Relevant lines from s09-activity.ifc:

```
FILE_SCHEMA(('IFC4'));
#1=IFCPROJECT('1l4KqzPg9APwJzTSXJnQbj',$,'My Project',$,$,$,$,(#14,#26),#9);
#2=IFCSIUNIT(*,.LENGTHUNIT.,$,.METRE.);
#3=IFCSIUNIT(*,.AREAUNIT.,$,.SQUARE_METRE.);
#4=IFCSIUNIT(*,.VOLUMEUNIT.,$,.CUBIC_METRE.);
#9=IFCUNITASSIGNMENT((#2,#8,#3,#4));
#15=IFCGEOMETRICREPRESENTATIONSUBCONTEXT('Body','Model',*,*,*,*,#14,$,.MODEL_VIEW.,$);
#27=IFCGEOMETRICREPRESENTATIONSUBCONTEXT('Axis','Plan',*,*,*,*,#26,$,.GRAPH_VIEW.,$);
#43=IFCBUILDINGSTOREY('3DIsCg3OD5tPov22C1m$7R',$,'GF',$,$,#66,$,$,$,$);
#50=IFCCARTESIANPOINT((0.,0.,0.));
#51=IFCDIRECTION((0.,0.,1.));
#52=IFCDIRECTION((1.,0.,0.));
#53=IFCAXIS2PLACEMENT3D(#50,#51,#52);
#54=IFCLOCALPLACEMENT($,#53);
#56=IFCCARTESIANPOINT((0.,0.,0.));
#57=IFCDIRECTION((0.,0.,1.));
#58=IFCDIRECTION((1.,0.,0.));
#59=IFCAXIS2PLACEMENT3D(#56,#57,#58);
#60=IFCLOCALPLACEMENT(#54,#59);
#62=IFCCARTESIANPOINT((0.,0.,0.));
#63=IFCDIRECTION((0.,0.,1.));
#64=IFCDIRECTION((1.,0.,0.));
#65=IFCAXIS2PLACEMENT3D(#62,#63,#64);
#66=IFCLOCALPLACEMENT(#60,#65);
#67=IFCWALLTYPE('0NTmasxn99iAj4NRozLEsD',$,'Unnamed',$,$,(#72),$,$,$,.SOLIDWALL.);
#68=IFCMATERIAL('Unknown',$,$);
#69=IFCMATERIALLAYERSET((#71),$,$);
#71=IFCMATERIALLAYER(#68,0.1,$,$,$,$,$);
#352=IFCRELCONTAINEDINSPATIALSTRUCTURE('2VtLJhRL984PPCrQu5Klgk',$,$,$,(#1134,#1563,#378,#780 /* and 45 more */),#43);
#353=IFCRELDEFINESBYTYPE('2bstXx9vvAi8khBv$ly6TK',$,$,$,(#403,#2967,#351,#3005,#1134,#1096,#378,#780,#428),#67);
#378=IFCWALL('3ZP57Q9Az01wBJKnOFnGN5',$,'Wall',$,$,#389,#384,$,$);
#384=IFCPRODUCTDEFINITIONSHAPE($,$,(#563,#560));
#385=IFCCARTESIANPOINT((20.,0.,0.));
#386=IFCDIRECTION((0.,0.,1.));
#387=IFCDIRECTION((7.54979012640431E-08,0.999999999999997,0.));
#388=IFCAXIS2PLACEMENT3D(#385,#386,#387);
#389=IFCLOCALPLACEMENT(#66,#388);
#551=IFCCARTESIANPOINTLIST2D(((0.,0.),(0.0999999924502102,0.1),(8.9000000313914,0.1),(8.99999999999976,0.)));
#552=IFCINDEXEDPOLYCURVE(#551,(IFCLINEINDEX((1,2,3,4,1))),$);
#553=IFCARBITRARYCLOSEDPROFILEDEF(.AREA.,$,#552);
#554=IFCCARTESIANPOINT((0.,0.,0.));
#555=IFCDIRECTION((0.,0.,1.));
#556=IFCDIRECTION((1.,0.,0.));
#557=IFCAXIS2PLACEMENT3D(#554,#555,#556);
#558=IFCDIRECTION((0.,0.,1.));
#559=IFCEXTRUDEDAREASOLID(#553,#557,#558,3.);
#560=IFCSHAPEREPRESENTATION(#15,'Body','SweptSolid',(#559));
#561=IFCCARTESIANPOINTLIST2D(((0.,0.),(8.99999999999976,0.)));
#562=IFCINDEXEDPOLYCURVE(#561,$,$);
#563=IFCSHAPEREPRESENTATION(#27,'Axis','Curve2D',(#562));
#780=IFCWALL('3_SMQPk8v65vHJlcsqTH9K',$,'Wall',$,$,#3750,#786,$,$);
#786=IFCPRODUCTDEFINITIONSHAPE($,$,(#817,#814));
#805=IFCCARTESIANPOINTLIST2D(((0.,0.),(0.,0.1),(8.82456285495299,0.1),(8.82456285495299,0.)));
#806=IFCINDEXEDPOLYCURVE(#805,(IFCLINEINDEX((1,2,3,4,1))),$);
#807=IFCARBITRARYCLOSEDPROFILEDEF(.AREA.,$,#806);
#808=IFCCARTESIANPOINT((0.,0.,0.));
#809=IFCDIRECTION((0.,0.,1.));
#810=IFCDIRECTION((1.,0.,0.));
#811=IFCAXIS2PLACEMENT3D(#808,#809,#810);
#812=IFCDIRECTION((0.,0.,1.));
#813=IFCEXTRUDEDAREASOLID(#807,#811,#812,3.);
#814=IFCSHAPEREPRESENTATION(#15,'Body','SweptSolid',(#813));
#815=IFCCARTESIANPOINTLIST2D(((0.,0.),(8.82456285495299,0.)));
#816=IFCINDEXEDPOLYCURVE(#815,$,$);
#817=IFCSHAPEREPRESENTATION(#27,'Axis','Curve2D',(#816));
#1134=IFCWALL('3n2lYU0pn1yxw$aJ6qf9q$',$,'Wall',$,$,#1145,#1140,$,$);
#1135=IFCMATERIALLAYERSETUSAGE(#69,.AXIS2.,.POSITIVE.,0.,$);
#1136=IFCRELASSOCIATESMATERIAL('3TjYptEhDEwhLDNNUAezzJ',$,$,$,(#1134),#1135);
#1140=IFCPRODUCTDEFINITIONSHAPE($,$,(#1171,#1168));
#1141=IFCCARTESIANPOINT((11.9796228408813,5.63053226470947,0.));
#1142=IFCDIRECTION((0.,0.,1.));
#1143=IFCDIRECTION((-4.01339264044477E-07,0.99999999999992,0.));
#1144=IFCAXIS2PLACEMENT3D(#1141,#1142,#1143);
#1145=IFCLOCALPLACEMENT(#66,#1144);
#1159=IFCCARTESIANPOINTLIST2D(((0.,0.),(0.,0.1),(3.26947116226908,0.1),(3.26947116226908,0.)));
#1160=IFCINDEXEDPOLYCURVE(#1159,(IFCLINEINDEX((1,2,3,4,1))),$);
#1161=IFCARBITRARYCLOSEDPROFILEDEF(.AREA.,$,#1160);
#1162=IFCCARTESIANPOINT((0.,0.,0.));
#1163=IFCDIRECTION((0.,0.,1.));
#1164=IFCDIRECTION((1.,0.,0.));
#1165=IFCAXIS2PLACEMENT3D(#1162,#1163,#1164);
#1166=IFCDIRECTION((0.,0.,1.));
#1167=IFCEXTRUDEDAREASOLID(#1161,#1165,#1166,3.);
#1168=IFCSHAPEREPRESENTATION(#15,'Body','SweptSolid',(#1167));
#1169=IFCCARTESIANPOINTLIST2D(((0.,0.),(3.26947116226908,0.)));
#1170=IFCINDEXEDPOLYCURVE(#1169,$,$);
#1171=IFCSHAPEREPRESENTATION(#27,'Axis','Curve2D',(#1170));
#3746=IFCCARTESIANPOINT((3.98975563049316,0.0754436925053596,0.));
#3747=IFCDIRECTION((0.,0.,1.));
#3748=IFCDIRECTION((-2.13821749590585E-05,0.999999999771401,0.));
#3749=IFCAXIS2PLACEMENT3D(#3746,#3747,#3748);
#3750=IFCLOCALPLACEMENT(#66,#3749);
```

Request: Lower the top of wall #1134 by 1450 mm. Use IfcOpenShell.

```python
import ifcopenshell
import ifcopenshell.geom
import ifcopenshell.util.representation
import ifcopenshell.util.shape
import ifcopenshell.util.unit

model = ifcopenshell.open("s09-activity.ifc")
unit_scale = ifcopenshell.util.unit.calculate_unit_scale(model)
settings = ifcopenshell.geom.settings()


def volume(element):
    """Net volume in cubic metres, openings subtracted."""
    shape = ifcopenshell.geom.create_shape(settings, element)
    return ifcopenshell.util.shape.get_volume(shape.geometry)


wall = model.by_guid("3n2lYU0pn1yxw$aJ6qf9q$")
before = volume(wall)

body = ifcopenshell.util.representation.get_representation(wall, "Model", "Body")
solid = body.Items[0]
old_height = solid.Depth
solid.Depth -= 1.45 / unit_scale
after = volume(wall)

print(f"height {old_height:g} -> {solid.Depth:g}, volume {before:.3f} -> {after:.3f} m3")

model.write("s09-activity_rev.ifc")
```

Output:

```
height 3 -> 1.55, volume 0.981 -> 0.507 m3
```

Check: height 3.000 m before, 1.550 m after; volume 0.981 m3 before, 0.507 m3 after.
